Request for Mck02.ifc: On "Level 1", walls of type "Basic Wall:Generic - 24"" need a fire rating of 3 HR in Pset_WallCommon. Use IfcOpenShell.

First a look at what the model holds.

```python
import ifcopenshell
import ifcopenshell.util.element

model = ifcopenshell.open("Mck02.ifc")
print(model.schema)
storey = next(s for s in model.by_type("IfcBuildingStorey") if s.Name == "Level 1")
walls = [e for e in ifcopenshell.util.element.get_decomposition(storey) if e.is_a("IfcWall")]
seen = {}
for e in walls:
    element_type = ifcopenshell.util.element.get_type(e)
    key = (element_type.Name if element_type != e and element_type else None, ifcopenshell.util.element.get_pset(e, "Pset_WallCommon", "FireRating"))
    seen[key] = seen.get(key, 0) + 1
for (name, value), count in sorted(seen.items(), key=str):
    print(count, "x", name, "|", value)
```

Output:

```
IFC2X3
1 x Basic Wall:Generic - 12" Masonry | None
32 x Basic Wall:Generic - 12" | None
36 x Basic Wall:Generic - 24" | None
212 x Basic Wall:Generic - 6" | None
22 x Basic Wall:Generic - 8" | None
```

```python
import ifcopenshell
import ifcopenshell.api.pset
import ifcopenshell.util.element

model = ifcopenshell.open("Mck02.ifc")

storey = next(s for s in model.by_type("IfcBuildingStorey") if s.Name == "Level 1")
walls = [e for e in ifcopenshell.util.element.get_decomposition(storey) if e.is_a("IfcWall")]

count = 0
for e in walls:
    element_type = ifcopenshell.util.element.get_type(e)
    if element_type in (None, e) or element_type.Name != 'Basic Wall:Generic - 24"':
        continue
    # add_pset returns the element's existing set when there is one.
    pset = ifcopenshell.api.pset.add_pset(model, product=e, name="Pset_WallCommon")
    ifcopenshell.api.pset.edit_pset(model, pset=pset, properties={"FireRating": "3 HR"})
    count += 1

print(count, "walls updated")

model.write("Mck02_rev.ifc")
```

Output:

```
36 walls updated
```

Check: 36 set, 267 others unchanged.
